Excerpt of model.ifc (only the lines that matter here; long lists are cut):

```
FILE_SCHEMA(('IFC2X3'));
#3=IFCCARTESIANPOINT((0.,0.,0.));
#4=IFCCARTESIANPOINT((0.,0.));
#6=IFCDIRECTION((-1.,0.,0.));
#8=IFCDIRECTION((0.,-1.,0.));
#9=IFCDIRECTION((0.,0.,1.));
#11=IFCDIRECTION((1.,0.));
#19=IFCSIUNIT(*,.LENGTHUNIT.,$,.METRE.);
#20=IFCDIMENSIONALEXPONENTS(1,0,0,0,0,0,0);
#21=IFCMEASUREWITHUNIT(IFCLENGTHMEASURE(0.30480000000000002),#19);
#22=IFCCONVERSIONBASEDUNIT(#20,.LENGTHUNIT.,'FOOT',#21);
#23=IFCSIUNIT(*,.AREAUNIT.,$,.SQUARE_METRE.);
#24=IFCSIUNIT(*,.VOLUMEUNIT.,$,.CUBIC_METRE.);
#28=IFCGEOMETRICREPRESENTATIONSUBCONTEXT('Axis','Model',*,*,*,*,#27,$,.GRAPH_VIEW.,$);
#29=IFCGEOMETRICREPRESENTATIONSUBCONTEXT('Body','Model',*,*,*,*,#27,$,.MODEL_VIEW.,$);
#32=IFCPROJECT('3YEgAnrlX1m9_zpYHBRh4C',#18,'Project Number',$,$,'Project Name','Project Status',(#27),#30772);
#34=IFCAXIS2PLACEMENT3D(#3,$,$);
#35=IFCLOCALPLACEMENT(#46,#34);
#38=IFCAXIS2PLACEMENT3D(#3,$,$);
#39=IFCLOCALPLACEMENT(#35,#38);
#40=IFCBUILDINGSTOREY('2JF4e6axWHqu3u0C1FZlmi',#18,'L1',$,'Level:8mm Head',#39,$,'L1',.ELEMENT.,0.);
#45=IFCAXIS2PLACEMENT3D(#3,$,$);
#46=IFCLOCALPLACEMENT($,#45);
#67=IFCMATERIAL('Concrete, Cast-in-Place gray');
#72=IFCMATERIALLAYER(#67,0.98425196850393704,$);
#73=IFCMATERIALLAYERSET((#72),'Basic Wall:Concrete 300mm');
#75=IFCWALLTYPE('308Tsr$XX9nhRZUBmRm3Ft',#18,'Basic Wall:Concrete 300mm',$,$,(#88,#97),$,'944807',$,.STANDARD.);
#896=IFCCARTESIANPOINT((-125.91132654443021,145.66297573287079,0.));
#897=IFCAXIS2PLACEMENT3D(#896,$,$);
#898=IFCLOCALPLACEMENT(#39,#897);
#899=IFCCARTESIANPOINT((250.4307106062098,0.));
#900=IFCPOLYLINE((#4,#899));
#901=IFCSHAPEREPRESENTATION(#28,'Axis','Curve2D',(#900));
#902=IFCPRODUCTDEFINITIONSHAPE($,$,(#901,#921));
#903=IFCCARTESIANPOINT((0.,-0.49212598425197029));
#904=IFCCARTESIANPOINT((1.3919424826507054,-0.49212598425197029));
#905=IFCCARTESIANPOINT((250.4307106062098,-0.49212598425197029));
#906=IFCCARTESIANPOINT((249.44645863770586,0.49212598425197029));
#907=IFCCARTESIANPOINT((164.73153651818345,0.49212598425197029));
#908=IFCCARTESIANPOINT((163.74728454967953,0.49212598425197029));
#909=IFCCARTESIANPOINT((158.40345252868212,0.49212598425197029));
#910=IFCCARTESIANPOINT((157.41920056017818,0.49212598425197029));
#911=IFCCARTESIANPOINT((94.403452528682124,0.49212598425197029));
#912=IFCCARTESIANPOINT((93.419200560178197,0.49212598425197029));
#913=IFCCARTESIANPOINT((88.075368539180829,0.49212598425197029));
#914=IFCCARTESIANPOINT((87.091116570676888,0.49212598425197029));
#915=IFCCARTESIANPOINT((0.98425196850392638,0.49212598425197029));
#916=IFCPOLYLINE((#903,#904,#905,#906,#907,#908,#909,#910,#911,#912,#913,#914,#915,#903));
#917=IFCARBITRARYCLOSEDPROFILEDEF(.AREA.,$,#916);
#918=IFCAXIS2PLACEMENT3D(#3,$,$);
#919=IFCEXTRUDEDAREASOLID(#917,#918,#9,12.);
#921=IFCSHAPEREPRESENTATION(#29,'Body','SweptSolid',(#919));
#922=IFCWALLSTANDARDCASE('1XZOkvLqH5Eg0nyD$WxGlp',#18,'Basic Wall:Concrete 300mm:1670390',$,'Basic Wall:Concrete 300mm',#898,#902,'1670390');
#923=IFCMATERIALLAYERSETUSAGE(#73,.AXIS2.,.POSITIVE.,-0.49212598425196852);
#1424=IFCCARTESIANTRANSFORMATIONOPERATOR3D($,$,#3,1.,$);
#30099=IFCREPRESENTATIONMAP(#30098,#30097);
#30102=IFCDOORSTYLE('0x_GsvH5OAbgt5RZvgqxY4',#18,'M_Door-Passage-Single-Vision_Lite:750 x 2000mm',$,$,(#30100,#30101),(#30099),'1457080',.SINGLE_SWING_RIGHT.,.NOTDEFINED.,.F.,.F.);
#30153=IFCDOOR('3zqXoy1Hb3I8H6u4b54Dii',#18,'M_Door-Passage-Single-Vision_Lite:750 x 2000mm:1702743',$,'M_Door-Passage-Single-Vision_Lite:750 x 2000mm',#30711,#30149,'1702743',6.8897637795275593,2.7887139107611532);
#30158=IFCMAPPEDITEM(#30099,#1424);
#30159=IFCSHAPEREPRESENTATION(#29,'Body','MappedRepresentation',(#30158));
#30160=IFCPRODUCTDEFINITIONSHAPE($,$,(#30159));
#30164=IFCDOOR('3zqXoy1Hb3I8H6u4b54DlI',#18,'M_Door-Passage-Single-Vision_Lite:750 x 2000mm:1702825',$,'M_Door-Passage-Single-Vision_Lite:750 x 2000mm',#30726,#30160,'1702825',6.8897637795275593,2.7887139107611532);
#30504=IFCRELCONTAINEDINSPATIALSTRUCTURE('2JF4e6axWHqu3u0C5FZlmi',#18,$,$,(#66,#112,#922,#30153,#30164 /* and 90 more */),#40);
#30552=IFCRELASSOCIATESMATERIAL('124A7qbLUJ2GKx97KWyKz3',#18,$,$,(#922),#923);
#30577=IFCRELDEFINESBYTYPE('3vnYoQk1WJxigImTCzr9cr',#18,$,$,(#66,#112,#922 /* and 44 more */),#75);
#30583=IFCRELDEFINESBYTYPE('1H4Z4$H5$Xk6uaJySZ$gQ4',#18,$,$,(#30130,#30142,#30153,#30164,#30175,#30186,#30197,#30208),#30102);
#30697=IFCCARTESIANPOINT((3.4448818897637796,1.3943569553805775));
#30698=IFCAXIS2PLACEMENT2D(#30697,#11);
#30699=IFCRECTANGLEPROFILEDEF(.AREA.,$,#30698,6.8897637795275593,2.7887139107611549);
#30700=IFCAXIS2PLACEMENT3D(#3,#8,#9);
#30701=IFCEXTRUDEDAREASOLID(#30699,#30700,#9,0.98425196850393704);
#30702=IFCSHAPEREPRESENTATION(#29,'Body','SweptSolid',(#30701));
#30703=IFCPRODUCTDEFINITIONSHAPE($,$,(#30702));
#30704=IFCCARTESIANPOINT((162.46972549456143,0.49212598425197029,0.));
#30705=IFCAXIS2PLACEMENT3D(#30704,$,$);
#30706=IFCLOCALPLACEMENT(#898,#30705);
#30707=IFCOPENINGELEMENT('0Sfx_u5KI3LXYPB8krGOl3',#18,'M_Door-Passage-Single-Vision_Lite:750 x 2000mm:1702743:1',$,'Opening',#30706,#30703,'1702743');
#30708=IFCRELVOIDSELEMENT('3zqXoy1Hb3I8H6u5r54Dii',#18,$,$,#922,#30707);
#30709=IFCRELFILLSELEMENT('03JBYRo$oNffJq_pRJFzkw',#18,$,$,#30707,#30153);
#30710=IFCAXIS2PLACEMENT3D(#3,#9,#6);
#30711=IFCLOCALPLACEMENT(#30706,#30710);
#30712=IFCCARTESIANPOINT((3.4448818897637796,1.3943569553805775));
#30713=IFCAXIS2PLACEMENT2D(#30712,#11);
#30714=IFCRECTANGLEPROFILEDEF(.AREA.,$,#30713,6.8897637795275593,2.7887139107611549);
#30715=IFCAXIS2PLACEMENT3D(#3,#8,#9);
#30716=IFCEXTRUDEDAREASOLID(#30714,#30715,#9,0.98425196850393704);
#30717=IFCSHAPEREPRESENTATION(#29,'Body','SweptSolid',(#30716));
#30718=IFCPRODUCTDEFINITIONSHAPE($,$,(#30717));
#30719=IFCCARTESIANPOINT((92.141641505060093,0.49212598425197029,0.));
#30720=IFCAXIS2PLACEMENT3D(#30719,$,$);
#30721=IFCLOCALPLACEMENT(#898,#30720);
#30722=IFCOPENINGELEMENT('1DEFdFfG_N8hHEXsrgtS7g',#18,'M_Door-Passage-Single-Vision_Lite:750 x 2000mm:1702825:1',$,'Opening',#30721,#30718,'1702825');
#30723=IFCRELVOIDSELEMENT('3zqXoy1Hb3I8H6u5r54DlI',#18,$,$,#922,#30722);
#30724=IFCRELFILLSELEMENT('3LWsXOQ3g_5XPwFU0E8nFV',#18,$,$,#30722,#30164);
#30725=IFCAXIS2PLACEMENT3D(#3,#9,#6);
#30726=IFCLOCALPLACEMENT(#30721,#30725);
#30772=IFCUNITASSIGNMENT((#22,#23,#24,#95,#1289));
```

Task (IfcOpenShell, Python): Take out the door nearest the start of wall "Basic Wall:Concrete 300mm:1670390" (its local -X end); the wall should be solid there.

```python
import ifcopenshell
import ifcopenshell.api.feature
import ifcopenshell.api.root
import ifcopenshell.geom
import ifcopenshell.util.shape

model = ifcopenshell.open("model.ifc")
settings = ifcopenshell.geom.settings()


def volume(element):
    """Net volume in cubic metres, openings subtracted."""
    shape = ifcopenshell.geom.create_shape(settings, element)
    return ifcopenshell.util.shape.get_volume(shape.geometry)


door = model.by_guid("3zqXoy1Hb3I8H6u4b54DlI")
opening = door.FillsVoids[0].RelatingOpeningElement
wall = opening.VoidsElements[0].RelatingBuildingElement
before = volume(wall)

ifcopenshell.api.root.remove_product(model, product=door)
ifcopenshell.api.feature.remove_feature(model, feature=opening)

after = volume(wall)

print(f"wall volume {before:.3f} -> {after:.3f} m3")

model.write("model_v2.ifc")
```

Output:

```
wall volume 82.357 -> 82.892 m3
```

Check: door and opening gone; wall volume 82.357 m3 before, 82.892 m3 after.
